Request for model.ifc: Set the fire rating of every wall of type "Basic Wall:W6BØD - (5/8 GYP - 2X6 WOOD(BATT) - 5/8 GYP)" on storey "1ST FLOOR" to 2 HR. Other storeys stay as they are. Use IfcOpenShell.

First a look at what the model holds.

```python
import ifcopenshell
import ifcopenshell.util.element

model = ifcopenshell.open("model.ifc")
print(model.schema)
storey = next(s for s in model.by_type("IfcBuildingStorey") if s.Name == "1ST FLOOR")
walls = [e for e in ifcopenshell.util.element.get_decomposition(storey) if e.is_a("IfcWall")]
seen = {}
for e in walls:
    element_type = ifcopenshell.util.element.get_type(e)
    key = (element_type.Name if element_type != e and element_type else None, ifcopenshell.util.element.get_pset(e, "Pset_WallCommon", "FireRating"))
    seen[key] = seen.get(key, 0) + 1
for (name, value), count in sorted(seen.items(), key=str):
    print(count, "x", name, "|", value)
```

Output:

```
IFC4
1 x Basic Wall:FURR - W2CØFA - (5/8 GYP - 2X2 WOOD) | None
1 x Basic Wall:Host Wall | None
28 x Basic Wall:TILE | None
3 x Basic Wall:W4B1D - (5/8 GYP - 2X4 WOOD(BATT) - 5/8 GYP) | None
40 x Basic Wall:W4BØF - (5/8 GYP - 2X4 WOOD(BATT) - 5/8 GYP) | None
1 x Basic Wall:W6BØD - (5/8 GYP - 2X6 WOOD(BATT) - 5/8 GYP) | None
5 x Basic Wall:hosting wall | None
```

```python
import ifcopenshell
import ifcopenshell.api.pset
import ifcopenshell.util.element

model = ifcopenshell.open("model.ifc")

storey = next(s for s in model.by_type("IfcBuildingStorey") if s.Name == "1ST FLOOR")
walls = [e for e in ifcopenshell.util.element.get_decomposition(storey) if e.is_a("IfcWall")]

count = 0
for e in walls:
    element_type = ifcopenshell.util.element.get_type(e)
    if element_type in (None, e) or element_type.Name != "Basic Wall:W6BØD - (5/8 GYP - 2X6 WOOD(BATT) - 5/8 GYP)":
        continue
    # add_pset returns the element's existing set when there is one.
    pset = ifcopenshell.api.pset.add_pset(model, product=e, name="Pset_WallCommon")
    ifcopenshell.api.pset.edit_pset(model, pset=pset, properties={"FireRating": "2 HR"})
    count += 1

print(count, "walls updated")

model.write("model_v2.ifc")
```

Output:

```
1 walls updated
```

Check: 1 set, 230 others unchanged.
